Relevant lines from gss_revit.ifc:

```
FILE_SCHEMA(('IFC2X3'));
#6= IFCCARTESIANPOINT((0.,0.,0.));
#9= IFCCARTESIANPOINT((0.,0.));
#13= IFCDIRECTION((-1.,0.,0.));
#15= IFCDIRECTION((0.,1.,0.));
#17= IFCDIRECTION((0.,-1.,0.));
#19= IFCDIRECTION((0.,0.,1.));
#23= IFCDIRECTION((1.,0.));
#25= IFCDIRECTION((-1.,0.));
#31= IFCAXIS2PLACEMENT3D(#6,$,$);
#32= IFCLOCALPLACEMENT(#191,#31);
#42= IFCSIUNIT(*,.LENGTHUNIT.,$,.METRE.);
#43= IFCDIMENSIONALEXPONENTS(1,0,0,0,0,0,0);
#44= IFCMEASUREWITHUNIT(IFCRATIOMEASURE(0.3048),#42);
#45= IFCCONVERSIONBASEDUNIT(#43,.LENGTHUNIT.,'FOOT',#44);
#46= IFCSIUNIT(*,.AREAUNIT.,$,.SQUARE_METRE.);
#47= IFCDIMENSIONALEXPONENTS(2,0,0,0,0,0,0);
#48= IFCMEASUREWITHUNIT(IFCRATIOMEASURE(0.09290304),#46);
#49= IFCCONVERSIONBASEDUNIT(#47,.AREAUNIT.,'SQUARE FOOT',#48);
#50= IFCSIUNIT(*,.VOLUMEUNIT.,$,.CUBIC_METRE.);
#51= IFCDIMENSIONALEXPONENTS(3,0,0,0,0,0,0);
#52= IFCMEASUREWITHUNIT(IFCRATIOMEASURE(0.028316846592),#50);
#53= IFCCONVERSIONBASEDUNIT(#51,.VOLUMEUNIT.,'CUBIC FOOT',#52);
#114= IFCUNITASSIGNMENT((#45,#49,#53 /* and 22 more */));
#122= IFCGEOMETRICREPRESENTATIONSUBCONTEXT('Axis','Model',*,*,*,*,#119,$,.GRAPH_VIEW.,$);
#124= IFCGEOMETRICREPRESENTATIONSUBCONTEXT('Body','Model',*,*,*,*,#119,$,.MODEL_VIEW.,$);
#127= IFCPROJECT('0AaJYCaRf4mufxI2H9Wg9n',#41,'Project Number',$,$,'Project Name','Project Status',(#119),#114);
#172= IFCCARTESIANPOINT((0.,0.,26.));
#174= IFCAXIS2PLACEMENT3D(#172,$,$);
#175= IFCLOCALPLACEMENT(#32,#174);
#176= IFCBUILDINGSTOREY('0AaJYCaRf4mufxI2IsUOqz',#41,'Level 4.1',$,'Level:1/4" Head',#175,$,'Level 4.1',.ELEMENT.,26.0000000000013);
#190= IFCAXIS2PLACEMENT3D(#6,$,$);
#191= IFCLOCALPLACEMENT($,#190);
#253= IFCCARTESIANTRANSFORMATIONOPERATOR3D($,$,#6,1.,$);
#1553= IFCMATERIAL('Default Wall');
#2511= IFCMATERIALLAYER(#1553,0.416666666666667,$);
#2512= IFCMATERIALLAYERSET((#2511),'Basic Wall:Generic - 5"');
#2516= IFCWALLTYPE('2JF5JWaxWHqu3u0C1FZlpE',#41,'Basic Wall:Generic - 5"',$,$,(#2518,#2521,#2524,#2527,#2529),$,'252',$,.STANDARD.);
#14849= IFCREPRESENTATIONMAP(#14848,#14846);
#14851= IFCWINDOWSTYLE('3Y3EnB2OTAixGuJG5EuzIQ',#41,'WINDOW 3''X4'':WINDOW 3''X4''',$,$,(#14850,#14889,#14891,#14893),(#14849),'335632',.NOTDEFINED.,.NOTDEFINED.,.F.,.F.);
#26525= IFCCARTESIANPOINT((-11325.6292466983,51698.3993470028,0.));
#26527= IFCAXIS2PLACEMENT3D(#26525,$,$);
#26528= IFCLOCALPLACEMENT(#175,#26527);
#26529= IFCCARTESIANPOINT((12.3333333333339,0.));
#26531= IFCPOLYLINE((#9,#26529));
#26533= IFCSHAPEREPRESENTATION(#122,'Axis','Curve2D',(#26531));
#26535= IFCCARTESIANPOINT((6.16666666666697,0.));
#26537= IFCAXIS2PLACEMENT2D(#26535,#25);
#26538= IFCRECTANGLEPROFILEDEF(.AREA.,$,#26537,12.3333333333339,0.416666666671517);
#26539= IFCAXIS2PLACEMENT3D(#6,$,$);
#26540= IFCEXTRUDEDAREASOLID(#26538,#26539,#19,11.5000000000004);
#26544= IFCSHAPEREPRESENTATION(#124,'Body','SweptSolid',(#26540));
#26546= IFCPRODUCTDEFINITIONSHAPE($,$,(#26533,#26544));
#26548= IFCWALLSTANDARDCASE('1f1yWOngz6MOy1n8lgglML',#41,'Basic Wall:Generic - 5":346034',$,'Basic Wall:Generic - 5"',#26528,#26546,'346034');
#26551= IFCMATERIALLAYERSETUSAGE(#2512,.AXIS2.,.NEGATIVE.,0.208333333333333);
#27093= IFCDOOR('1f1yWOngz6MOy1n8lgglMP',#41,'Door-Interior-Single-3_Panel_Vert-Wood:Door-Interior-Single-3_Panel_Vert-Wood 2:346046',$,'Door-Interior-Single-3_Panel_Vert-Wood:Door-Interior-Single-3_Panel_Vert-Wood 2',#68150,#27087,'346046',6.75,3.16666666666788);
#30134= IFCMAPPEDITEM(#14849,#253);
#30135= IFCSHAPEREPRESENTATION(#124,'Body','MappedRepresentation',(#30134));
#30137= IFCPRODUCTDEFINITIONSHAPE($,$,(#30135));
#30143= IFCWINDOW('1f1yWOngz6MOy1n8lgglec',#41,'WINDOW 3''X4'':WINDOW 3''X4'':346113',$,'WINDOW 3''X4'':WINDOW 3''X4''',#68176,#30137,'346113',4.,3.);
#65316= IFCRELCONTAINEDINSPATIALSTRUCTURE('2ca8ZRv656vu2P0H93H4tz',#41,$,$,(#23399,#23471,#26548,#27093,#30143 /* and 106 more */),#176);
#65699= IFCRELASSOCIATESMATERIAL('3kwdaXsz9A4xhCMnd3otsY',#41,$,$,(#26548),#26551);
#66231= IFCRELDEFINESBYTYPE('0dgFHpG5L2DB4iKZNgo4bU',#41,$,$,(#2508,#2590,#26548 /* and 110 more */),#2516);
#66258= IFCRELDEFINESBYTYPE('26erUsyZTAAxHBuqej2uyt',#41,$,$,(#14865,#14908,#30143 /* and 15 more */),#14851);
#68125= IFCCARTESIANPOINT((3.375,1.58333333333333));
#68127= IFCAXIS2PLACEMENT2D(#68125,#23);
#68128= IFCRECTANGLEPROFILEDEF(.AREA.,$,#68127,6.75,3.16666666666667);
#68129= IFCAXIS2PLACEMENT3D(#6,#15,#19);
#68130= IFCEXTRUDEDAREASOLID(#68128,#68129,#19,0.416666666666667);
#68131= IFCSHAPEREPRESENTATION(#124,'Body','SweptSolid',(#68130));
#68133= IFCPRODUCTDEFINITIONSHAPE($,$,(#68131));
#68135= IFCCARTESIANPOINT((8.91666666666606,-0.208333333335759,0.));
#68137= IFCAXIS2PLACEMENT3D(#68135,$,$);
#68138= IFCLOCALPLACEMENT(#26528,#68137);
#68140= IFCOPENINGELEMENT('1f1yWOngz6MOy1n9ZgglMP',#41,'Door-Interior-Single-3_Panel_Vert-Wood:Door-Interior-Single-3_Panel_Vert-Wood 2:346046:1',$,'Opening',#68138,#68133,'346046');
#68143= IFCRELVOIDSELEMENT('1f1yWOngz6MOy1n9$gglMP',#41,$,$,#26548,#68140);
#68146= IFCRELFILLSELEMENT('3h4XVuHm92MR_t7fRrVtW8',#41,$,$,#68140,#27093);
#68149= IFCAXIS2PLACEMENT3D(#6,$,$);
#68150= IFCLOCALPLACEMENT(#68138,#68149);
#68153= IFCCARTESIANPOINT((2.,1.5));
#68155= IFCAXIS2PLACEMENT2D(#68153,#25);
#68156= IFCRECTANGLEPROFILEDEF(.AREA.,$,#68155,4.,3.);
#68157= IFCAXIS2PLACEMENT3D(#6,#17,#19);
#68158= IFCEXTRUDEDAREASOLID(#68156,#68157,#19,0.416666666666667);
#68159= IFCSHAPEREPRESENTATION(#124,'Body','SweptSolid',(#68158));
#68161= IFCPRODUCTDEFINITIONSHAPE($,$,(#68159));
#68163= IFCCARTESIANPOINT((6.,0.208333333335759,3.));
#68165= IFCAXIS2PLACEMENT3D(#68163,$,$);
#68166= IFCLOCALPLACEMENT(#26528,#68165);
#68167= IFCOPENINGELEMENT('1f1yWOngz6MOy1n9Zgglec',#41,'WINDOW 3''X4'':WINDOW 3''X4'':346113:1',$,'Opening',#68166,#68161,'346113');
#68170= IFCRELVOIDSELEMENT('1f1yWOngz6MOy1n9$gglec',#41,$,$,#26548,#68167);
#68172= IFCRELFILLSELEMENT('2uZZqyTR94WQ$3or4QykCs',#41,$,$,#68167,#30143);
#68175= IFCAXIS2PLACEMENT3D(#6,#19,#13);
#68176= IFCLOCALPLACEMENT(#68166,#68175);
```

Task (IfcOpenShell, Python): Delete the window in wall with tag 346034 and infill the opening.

```python
import ifcopenshell
import ifcopenshell.api.feature
import ifcopenshell.api.root
import ifcopenshell.geom
import ifcopenshell.util.shape

model = ifcopenshell.open("gss_revit.ifc")
settings = ifcopenshell.geom.settings()


def volume(element):
    """Net volume in cubic metres, openings subtracted."""
    shape = ifcopenshell.geom.create_shape(settings, element)
    return ifcopenshell.util.shape.get_volume(shape.geometry)


window = model.by_id(30143)
opening = window.FillsVoids[0].RelatingOpeningElement
wall = opening.VoidsElements[0].RelatingBuildingElement
before = volume(wall)

ifcopenshell.api.root.remove_product(model, product=window)
ifcopenshell.api.feature.remove_feature(model, feature=opening)

after = volume(wall)

print(f"wall volume {before:.3f} -> {after:.3f} m3")

model.write("gss_revit_edited.ifc")
```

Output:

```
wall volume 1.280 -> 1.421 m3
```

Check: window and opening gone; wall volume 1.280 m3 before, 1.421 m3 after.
